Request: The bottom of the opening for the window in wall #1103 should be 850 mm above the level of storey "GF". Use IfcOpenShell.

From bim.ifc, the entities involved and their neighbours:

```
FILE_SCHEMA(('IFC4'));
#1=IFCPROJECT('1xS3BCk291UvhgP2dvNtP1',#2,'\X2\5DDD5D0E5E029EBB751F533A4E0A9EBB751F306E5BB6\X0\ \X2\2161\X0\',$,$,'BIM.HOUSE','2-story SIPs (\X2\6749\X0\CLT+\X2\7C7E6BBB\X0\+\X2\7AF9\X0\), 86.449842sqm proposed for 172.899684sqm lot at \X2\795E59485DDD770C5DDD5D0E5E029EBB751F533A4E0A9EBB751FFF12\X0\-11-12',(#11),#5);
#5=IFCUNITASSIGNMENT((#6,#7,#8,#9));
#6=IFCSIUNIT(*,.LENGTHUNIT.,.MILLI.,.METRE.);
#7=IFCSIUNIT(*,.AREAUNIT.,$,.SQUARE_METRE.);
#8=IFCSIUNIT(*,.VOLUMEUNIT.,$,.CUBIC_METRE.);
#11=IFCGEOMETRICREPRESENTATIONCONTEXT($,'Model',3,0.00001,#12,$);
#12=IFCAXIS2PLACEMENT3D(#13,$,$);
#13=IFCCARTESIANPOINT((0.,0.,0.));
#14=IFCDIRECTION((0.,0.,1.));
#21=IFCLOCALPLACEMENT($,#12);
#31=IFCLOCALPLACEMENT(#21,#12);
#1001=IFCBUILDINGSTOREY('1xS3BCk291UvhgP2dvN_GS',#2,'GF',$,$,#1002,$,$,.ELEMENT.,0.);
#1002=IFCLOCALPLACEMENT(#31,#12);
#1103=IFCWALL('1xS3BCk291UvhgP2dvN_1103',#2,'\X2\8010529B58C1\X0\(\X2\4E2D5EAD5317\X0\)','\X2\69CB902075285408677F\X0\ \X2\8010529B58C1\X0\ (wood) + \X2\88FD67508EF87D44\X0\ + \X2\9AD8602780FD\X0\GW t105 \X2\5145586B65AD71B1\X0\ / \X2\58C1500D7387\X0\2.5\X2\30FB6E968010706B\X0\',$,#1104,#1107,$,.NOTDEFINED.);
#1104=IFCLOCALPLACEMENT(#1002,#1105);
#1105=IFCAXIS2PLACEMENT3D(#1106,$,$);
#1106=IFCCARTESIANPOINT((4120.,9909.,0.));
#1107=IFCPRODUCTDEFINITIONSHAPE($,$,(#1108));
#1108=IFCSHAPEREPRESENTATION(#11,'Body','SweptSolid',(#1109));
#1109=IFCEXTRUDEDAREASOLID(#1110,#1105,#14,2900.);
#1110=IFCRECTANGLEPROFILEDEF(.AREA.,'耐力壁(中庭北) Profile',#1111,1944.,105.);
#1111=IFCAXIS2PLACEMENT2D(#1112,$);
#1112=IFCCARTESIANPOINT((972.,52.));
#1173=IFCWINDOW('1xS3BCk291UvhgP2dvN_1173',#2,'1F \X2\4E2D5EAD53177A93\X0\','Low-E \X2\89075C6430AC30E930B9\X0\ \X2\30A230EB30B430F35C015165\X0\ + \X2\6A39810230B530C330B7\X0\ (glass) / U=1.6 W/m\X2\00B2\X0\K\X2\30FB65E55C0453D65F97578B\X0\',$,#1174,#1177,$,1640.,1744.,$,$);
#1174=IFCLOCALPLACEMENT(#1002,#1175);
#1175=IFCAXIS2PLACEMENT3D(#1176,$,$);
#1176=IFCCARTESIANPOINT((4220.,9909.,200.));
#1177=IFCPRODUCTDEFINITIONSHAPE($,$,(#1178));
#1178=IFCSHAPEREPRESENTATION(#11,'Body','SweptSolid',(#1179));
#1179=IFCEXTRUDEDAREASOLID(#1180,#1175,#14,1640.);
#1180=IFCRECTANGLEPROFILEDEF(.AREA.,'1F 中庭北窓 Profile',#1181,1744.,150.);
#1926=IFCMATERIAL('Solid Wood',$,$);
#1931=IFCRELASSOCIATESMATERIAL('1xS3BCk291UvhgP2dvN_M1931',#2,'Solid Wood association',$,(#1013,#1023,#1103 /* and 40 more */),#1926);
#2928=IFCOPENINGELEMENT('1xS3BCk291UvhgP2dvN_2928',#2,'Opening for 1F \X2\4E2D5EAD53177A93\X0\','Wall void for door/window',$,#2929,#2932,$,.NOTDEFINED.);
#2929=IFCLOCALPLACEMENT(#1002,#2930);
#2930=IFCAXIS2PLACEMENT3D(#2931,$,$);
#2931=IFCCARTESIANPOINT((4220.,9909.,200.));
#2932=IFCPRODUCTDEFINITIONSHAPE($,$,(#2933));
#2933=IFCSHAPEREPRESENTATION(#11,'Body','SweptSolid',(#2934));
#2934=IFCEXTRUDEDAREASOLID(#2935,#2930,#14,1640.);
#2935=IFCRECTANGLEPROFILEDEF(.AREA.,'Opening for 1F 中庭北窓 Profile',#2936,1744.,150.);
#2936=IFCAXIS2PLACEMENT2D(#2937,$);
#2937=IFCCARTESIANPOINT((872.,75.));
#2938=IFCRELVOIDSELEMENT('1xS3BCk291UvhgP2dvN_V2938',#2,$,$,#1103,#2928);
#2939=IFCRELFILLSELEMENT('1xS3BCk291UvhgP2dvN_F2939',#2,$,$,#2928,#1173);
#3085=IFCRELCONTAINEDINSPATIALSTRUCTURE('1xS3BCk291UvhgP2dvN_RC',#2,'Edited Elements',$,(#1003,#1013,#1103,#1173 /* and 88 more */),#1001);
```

```python
import numpy as np
import ifcopenshell
import ifcopenshell.api.geometry
import ifcopenshell.geom
import ifcopenshell.util.element
import ifcopenshell.util.placement
import ifcopenshell.util.shape
import ifcopenshell.util.unit

model = ifcopenshell.open("bim.ifc")
unit_scale = ifcopenshell.util.unit.calculate_unit_scale(model)

window = model.by_guid("1xS3BCk291UvhgP2dvN_1173")
opening = window.FillsVoids[0].RelatingOpeningElement
storey = ifcopenshell.util.element.get_container(window, ifc_class="IfcBuildingStorey")
level = ifcopenshell.util.placement.get_local_placement(storey.ObjectPlacement)[2, 3]

# The opening's origin need not be at the sill, so measure its lowest point.
shape = ifcopenshell.geom.create_shape(ifcopenshell.geom.settings(), opening)
bottom = ifcopenshell.util.shape.get_shape_bottom_elevation(shape, shape.geometry) / unit_scale
dz = level + 850.0 - bottom

shift = np.array([0.0, 0.0, dz])
# The window is not placed relative to its opening, so move both.
for product in (opening, window):
    matrix = ifcopenshell.util.placement.get_local_placement(product.ObjectPlacement)
    matrix[:3, 3] += shift
    ifcopenshell.api.geometry.edit_object_placement(model, product=product, matrix=matrix, is_si=False)

print(f"moved by {dz * unit_scale:+.3f} m")

model.write("bim_rev.ifc")
```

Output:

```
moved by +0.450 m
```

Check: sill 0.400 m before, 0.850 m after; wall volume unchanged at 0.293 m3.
